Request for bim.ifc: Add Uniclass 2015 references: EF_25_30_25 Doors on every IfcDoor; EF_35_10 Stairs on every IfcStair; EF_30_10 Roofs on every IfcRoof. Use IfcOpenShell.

First a look at what the model holds.

```python
import ifcopenshell

model = ifcopenshell.open("bim.ifc")
print(model.schema)
print("classifications:", [c.Name for c in model.by_type("IfcClassification")])
for ifc_class in ("IfcDoor", "IfcRoof", "IfcStair", "IfcWall", "IfcWindow"):
    print(ifc_class, len(model.by_type(ifc_class)))
```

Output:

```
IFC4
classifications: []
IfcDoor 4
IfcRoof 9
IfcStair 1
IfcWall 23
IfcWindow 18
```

```python
import ifcopenshell
import ifcopenshell.api.classification

model = ifcopenshell.open("bim.ifc")

system = ifcopenshell.api.classification.add_classification(model, classification="Uniclass 2015")

codes = {
    "IfcDoor": ("EF_25_30_25", "Doors"),
    "IfcStair": ("EF_35_10", "Stairs"),
    "IfcRoof": ("EF_30_10", "Roofs"),
}
for ifc_class, (code, name) in codes.items():
    products = model.by_type(ifc_class)
    ifcopenshell.api.classification.add_reference(
        model, products=products, classification=system, identification=code, name=name
    )
    print(code, len(products))

model.write("bim-out.ifc")
```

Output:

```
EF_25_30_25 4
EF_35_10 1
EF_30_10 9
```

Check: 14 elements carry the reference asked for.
